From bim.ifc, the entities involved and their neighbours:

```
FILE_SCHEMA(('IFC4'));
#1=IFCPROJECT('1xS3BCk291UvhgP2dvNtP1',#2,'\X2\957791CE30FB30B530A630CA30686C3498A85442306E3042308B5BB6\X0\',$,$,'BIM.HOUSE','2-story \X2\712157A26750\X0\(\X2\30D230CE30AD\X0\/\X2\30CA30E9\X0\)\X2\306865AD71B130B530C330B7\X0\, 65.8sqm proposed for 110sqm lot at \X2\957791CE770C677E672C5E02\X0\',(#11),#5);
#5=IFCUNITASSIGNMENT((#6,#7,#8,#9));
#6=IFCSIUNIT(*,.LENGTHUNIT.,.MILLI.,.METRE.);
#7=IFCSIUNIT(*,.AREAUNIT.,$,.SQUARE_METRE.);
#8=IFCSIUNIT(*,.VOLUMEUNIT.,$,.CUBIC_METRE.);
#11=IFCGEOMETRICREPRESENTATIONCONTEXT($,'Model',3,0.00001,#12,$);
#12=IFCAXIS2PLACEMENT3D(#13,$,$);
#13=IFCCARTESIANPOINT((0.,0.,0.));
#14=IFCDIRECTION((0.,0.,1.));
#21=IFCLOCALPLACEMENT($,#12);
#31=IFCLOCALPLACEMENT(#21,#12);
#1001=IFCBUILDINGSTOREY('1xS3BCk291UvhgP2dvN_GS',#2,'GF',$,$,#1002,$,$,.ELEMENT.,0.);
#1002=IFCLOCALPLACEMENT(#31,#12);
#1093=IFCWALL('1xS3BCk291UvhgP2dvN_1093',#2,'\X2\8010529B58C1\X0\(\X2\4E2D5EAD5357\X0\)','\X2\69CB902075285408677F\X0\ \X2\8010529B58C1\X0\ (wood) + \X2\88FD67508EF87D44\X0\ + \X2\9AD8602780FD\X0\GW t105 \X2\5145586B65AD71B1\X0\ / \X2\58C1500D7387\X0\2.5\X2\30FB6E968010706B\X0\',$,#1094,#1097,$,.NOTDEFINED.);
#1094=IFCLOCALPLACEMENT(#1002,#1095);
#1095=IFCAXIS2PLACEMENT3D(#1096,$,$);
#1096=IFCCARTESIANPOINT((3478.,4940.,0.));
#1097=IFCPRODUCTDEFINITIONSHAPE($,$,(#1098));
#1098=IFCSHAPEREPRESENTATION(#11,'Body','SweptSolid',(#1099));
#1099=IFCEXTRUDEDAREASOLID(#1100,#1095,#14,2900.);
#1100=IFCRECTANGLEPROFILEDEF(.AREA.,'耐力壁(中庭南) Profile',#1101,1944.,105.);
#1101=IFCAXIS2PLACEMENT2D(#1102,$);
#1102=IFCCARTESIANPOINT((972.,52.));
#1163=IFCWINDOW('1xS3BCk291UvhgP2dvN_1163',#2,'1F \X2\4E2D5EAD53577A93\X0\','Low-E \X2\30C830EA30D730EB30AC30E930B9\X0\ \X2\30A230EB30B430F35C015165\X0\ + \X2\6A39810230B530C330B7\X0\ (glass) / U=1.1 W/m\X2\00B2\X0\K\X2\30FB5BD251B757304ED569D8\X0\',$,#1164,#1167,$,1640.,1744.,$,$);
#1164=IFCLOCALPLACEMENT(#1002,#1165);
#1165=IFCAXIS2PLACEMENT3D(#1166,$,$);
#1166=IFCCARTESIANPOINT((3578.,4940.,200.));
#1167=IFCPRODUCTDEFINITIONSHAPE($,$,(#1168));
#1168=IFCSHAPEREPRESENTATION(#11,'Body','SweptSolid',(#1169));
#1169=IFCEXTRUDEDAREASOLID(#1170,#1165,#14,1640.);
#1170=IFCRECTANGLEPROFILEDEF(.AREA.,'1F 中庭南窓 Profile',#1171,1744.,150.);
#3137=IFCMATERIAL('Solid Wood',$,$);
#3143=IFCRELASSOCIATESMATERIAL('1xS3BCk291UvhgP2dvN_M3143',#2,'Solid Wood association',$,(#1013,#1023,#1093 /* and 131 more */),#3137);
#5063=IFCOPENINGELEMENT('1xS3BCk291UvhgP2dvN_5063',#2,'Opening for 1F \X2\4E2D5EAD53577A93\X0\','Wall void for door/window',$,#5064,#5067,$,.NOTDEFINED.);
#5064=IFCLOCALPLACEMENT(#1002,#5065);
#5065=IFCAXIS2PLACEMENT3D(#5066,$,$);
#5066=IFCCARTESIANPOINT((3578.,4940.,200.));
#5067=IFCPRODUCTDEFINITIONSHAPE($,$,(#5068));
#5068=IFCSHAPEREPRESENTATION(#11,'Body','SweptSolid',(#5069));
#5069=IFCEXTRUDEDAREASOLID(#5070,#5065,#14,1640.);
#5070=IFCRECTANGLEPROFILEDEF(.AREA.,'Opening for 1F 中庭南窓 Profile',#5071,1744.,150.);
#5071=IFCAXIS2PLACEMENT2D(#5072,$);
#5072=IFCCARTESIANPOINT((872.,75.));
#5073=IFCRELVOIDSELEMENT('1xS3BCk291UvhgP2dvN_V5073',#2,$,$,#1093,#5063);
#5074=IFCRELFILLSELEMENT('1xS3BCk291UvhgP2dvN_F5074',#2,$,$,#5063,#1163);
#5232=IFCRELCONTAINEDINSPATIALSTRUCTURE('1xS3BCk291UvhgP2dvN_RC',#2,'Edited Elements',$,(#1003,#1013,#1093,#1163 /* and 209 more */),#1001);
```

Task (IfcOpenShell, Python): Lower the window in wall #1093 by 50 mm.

```python
import numpy as np
import ifcopenshell
import ifcopenshell.api.geometry
import ifcopenshell.util.placement
import ifcopenshell.util.unit

model = ifcopenshell.open("bim.ifc")
unit_scale = ifcopenshell.util.unit.calculate_unit_scale(model)

window = model.by_guid("1xS3BCk291UvhgP2dvN_1163")
opening = window.FillsVoids[0].RelatingOpeningElement
dz = -50.0

shift = np.array([0.0, 0.0, dz])
# The window is not placed relative to its opening, so move both.
for product in (opening, window):
    matrix = ifcopenshell.util.placement.get_local_placement(product.ObjectPlacement)
    matrix[:3, 3] += shift
    ifcopenshell.api.geometry.edit_object_placement(model, product=product, matrix=matrix, is_si=False)

print(f"moved by {dz * unit_scale:+.3f} m")

model.write("bim_v2.ifc")
```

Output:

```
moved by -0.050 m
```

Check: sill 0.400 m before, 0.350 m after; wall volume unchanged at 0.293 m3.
